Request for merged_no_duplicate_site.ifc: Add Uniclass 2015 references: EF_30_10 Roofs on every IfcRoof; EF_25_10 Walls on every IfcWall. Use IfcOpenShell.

First a look at what the model holds.

```python
import ifcopenshell

model = ifcopenshell.open("merged_no_duplicate_site.ifc")
print(model.schema)
print("classifications:", [c.Name for c in model.by_type("IfcClassification")])
for ifc_class in ("IfcDoor", "IfcRoof", "IfcStair", "IfcWall", "IfcWindow"):
    print(ifc_class, len(model.by_type(ifc_class)))
```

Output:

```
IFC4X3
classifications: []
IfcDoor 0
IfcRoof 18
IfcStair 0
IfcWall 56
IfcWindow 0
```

```python
import ifcopenshell
import ifcopenshell.api.classification

model = ifcopenshell.open("merged_no_duplicate_site.ifc")

system = ifcopenshell.api.classification.add_classification(model, classification="Uniclass 2015")

codes = {
    "IfcRoof": ("EF_30_10", "Roofs"),
    "IfcWall": ("EF_25_10", "Walls"),
}
for ifc_class, (code, name) in codes.items():
    products = model.by_type(ifc_class)
    ifcopenshell.api.classification.add_reference(
        model, products=products, classification=system, identification=code, name=name
    )
    print(code, len(products))

model.write("merged_no_duplicate_site-out.ifc")
```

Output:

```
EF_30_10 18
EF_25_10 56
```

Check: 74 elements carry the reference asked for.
